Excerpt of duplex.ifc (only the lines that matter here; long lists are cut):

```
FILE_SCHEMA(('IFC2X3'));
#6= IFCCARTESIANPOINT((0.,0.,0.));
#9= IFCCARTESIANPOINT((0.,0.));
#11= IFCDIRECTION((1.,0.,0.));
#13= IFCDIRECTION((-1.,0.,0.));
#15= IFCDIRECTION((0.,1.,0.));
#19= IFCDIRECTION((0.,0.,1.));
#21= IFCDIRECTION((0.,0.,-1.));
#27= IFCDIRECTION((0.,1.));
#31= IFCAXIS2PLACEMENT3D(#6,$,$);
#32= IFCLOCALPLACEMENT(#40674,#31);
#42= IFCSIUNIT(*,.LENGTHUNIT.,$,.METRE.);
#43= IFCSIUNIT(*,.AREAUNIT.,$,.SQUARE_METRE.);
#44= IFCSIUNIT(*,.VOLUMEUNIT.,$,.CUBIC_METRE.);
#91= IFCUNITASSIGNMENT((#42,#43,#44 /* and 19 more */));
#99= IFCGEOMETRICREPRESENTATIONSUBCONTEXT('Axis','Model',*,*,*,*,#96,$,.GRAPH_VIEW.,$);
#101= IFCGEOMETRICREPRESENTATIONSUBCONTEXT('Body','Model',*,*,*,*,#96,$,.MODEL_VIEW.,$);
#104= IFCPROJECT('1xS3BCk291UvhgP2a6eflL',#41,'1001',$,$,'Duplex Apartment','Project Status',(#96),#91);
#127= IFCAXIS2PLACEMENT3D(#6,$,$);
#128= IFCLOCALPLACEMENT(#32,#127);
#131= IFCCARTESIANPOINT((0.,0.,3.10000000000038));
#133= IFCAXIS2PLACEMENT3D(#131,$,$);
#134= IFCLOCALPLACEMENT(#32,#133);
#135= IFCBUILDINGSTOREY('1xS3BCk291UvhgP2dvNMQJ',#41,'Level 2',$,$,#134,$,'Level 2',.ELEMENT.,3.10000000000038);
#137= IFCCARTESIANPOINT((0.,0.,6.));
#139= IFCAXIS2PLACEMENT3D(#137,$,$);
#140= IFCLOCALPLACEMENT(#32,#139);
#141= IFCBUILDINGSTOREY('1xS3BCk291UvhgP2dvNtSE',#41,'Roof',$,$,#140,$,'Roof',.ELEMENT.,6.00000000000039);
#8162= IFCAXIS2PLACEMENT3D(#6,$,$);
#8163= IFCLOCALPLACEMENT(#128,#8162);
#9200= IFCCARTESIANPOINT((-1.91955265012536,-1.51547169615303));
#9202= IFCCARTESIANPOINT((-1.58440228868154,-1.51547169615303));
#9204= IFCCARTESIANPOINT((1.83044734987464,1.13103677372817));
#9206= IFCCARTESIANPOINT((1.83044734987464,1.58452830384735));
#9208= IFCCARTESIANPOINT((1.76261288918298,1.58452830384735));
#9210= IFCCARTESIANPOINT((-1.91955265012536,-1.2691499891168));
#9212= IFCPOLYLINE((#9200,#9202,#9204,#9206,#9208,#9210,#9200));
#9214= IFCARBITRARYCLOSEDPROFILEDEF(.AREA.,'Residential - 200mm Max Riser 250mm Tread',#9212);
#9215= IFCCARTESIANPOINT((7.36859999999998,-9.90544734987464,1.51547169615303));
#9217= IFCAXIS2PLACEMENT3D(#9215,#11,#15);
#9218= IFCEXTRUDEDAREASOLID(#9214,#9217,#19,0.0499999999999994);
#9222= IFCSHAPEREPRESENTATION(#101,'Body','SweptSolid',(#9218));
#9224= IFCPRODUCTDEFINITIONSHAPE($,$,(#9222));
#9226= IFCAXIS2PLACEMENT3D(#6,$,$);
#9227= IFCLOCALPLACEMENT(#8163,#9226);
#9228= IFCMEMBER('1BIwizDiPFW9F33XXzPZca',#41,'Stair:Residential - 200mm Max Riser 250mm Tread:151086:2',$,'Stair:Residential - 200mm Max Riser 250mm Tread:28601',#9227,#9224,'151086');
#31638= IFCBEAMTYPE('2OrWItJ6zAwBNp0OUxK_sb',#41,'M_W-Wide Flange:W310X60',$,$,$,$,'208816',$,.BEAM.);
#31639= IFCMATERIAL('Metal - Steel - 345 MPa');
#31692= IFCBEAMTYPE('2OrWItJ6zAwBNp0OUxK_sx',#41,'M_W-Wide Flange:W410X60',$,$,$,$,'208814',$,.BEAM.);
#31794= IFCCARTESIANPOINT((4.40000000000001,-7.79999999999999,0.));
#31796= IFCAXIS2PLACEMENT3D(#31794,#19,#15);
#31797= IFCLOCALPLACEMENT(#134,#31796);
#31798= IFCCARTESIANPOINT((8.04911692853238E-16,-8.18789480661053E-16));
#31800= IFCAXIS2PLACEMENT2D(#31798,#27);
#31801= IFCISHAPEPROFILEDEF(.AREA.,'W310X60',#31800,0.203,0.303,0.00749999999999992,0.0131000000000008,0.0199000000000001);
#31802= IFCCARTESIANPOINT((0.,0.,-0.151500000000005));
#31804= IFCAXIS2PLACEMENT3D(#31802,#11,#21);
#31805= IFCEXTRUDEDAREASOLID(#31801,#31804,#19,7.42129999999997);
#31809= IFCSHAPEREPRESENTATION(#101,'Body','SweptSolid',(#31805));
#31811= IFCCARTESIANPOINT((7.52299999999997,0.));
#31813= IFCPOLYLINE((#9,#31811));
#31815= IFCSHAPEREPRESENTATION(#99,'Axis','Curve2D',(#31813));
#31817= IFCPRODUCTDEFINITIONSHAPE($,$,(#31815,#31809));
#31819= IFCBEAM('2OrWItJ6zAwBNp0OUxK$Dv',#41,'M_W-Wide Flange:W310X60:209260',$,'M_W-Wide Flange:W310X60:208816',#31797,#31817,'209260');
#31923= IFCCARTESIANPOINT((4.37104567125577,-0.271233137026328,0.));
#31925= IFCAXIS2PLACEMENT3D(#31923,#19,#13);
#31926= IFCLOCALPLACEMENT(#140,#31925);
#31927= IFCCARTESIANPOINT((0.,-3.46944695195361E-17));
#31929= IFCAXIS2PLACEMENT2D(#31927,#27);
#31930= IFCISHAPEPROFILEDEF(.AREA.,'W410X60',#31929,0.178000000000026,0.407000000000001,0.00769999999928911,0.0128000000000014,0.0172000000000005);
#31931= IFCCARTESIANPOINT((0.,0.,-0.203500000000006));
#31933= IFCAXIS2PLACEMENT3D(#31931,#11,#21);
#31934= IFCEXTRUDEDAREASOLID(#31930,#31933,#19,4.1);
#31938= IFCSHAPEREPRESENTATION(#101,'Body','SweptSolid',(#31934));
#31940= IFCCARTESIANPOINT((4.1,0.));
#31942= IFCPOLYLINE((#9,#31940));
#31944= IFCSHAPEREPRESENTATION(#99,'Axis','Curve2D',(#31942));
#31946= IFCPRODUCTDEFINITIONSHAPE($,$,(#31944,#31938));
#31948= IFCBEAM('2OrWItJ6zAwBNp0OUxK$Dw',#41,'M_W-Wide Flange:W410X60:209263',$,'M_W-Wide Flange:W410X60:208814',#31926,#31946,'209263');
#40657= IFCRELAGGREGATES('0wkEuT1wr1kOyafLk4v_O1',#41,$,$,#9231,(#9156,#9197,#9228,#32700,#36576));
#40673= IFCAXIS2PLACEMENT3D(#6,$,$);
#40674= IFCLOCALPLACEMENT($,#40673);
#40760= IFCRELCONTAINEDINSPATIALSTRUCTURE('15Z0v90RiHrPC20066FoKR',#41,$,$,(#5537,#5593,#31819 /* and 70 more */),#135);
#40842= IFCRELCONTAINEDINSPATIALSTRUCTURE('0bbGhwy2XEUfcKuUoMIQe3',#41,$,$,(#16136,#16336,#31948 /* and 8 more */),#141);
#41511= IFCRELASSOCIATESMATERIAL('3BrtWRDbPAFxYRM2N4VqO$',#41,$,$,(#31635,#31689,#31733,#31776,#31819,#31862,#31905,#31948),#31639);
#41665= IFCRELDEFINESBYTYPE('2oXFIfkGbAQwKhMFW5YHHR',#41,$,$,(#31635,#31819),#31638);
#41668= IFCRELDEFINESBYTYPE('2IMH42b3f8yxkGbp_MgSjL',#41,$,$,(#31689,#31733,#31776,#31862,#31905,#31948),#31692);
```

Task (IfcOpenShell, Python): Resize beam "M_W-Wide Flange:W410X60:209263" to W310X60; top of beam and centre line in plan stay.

```python
import ifcopenshell
import ifcopenshell.api.type
import ifcopenshell.util.element
import ifcopenshell.util.representation

model = ifcopenshell.open("duplex.ifc")

member = model.by_id(31948)
source = next(p for p in model.by_type("IfcIShapeProfileDef") if p.ProfileName == "W310X60")

body = ifcopenshell.util.representation.get_representation(member, "Model", "Body")
solid = body.Items[0]
old_profile = solid.SweptArea

# Copy the section's sizes but keep this member's own profile position.
profile = ifcopenshell.util.element.copy(model, source)
# Profiles are centred, so shift by half the change in depth to hold the top.
shift = (old_profile.OverallDepth - profile.OverallDepth) / 2
x, y = old_profile.Position.Location.Coordinates
up = (-1.0, 0.0)  # upwards, in the solid's own plane
location = model.createIfcCartesianPoint((x + up[0] * shift, y + up[1] * shift))
profile.Position = model.createIfcAxis2Placement2D(location, old_profile.Position.RefDirection)
solid.SweptArea = profile
if not model.get_total_inverses(old_profile):
    ifcopenshell.util.element.remove_deep2(model, old_profile)

new_type = model.by_guid("2OrWItJ6zAwBNp0OUxK_sb")
ifcopenshell.api.type.assign_type(
    model, related_objects=[member], relating_type=new_type, should_map_representations=False
)
member.Name = member.Name.replace("W410X60", "W310X60")
member.ObjectType = "M_W-Wide Flange:W310X60:208814"

print(solid.SweptArea)

model.write("duplex_v2.ifc")
```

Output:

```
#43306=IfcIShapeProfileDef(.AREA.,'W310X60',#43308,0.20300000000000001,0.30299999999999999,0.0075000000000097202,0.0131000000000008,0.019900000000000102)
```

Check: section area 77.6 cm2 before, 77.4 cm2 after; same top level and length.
